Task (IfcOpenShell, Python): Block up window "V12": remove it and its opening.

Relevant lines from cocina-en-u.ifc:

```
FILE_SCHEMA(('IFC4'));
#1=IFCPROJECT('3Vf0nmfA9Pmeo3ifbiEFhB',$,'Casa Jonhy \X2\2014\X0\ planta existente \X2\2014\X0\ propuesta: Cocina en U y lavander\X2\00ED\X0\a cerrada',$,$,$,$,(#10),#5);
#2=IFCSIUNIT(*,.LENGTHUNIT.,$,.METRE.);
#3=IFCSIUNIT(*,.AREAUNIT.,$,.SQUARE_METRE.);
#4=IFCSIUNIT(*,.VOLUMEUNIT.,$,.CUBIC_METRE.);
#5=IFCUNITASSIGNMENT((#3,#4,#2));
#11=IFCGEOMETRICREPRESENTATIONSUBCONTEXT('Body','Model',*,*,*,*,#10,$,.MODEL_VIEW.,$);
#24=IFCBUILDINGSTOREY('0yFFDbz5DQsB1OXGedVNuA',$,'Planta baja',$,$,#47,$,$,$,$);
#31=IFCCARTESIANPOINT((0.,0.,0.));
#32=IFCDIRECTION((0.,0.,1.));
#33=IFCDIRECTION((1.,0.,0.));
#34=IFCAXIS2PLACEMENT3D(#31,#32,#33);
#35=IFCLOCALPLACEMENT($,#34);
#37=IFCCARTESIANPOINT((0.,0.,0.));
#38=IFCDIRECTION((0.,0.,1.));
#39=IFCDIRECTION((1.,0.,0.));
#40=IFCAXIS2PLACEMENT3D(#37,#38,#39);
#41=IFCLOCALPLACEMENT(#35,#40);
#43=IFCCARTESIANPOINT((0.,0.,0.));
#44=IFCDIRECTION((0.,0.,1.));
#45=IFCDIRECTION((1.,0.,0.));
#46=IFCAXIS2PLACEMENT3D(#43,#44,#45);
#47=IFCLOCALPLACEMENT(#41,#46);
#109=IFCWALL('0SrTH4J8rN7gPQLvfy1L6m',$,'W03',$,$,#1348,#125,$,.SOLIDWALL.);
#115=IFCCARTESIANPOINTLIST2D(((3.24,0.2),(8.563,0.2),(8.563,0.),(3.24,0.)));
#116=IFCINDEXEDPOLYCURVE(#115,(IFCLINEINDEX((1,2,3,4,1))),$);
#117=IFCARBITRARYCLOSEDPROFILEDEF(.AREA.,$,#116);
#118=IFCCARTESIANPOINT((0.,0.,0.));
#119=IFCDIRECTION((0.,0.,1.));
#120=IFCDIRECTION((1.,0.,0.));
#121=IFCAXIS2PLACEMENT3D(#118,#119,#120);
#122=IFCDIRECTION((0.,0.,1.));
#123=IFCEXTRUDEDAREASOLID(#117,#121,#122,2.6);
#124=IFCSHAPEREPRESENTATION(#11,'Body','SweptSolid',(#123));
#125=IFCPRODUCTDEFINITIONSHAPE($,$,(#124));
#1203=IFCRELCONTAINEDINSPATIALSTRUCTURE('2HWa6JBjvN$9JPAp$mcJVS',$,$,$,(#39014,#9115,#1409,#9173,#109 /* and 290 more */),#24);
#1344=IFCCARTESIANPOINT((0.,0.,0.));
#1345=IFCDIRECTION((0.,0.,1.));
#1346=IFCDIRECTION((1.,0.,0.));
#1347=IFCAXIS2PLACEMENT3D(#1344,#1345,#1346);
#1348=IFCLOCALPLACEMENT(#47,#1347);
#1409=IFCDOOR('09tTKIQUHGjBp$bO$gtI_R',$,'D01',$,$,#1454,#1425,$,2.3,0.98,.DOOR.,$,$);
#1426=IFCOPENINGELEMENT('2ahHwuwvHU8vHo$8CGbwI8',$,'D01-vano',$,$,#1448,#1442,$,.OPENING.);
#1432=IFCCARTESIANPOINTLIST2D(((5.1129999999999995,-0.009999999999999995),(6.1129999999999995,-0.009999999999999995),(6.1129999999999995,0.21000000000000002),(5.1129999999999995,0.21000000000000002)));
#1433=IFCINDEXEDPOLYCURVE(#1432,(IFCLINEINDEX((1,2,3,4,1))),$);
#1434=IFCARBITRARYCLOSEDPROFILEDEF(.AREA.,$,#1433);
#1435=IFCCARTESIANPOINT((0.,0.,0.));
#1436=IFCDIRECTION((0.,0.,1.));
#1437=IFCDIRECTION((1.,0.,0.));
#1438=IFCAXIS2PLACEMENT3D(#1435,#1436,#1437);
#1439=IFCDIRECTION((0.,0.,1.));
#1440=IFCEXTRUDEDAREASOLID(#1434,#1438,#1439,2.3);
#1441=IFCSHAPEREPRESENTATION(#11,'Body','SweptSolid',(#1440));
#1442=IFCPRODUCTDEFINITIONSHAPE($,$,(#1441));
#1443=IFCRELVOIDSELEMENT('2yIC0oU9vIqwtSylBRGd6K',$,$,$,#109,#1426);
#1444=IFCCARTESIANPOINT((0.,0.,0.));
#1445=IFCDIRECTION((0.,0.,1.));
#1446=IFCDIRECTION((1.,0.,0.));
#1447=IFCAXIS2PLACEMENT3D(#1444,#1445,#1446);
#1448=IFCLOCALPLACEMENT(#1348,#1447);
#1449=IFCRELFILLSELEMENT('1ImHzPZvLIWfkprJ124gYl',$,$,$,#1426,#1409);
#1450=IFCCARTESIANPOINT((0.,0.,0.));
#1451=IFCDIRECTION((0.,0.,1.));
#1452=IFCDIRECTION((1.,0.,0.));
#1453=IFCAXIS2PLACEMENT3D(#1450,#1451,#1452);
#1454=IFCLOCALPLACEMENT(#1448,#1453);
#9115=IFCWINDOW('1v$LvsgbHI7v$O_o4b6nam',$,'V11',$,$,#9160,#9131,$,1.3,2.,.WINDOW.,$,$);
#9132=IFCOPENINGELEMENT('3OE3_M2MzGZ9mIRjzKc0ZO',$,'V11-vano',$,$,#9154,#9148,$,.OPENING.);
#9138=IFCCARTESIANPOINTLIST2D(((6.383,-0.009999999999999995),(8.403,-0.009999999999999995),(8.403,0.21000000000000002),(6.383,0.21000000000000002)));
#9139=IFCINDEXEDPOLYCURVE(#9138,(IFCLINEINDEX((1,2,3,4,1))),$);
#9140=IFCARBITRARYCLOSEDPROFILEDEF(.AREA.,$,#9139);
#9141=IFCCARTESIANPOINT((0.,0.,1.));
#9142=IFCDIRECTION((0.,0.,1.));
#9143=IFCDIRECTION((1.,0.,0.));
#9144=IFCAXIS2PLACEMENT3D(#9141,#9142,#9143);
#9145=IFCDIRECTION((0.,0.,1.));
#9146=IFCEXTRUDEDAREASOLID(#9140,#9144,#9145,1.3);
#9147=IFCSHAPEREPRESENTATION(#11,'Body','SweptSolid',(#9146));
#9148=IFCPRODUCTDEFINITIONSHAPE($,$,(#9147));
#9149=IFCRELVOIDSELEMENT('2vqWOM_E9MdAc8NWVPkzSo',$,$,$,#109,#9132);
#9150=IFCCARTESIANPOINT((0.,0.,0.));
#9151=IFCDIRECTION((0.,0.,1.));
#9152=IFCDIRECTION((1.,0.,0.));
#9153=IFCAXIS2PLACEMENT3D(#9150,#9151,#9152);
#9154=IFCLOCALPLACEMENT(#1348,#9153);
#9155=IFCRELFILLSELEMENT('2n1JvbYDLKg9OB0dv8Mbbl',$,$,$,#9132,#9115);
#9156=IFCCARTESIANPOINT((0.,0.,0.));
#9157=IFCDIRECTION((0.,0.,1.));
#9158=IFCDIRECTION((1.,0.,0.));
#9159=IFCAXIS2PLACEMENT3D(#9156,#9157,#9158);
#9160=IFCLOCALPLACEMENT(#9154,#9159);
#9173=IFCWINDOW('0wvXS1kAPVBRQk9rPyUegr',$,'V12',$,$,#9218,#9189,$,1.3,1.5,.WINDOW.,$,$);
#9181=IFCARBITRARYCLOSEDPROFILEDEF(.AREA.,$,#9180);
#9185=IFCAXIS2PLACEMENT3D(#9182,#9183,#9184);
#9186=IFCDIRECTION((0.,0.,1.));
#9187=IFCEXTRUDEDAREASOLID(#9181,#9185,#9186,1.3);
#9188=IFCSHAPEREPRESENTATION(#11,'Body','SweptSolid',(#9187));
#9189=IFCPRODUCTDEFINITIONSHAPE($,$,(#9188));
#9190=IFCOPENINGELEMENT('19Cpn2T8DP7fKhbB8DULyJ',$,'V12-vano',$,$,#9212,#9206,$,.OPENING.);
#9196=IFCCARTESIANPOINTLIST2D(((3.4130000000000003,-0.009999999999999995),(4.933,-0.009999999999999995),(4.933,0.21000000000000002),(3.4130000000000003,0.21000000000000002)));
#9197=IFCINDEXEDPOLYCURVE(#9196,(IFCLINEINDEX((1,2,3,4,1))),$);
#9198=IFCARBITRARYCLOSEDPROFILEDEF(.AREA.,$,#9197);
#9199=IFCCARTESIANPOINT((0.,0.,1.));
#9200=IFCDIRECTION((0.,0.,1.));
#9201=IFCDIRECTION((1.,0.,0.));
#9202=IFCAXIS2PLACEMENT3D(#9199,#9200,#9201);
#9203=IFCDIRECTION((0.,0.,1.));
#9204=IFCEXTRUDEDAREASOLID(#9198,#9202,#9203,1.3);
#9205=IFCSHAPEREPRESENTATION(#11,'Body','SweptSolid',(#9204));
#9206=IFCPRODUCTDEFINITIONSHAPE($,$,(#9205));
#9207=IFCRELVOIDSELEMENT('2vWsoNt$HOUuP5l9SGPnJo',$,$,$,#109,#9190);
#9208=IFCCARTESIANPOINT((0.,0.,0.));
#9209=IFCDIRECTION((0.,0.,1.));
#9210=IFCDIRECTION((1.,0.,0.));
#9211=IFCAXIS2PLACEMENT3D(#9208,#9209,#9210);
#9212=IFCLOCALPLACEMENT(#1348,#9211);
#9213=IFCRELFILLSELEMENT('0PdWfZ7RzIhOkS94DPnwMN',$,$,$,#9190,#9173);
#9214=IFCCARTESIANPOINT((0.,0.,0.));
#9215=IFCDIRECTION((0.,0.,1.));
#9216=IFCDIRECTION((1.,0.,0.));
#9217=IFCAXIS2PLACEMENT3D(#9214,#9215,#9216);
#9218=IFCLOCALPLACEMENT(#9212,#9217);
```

```python
import ifcopenshell
import ifcopenshell.api.feature
import ifcopenshell.api.root
import ifcopenshell.geom
import ifcopenshell.util.shape

model = ifcopenshell.open("cocina-en-u.ifc")
settings = ifcopenshell.geom.settings()


def volume(element):
    """Net volume in cubic metres, openings subtracted."""
    shape = ifcopenshell.geom.create_shape(settings, element)
    return ifcopenshell.util.shape.get_volume(shape.geometry)


window = model.by_guid("0wvXS1kAPVBRQk9rPyUegr")
opening = window.FillsVoids[0].RelatingOpeningElement
wall = opening.VoidsElements[0].RelatingBuildingElement
before = volume(wall)

ifcopenshell.api.root.remove_product(model, product=window)
ifcopenshell.api.feature.remove_feature(model, feature=opening)

after = volume(wall)

print(f"wall volume {before:.3f} -> {after:.3f} m3")

model.write("cocina-en-u-out.ifc")
```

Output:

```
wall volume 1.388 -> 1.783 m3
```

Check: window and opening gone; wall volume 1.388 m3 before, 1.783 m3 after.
